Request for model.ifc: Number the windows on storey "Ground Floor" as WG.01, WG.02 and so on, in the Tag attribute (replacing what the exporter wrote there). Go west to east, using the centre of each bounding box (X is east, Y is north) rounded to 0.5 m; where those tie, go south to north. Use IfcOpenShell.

First a look at what the model holds.

```python
import ifcopenshell
import ifcopenshell.util.element
import ifcopenshell.util.placement

model = ifcopenshell.open("model.ifc")
print(model.schema)
storey = next(s for s in model.by_type("IfcBuildingStorey") if s.Name == "Ground Floor")
windows = [e for e in ifcopenshell.util.element.get_decomposition(storey) if e.is_a("IfcWindow")]
for e in sorted(windows, key=lambda e: e.id()):
    origin = ifcopenshell.util.placement.get_local_placement(e.ObjectPlacement)[:3, 3]
    print(e.id(), e.Tag, e.Name, origin.round(2) + 0.0, sep=" | ")
```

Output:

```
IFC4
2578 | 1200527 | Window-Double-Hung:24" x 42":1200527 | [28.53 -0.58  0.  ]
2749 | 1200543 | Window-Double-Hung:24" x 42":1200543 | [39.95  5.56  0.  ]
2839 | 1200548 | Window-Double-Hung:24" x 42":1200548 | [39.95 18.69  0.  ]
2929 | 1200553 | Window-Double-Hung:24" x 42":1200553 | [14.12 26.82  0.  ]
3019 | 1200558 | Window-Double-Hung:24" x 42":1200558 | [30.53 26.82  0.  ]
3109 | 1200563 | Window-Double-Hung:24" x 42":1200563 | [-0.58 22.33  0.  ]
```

```python
import ifcopenshell
import ifcopenshell.geom
import ifcopenshell.util.element
import ifcopenshell.util.shape

model = ifcopenshell.open("model.ifc")
settings = ifcopenshell.geom.settings()
settings.set("use-world-coords", True)


def centre(element):
    shape = ifcopenshell.geom.create_shape(settings, element)
    return ifcopenshell.util.shape.get_bbox_centroid(shape.geometry)


storey = next(s for s in model.by_type("IfcBuildingStorey") if s.Name == "Ground Floor")
windows = [e for e in ifcopenshell.util.element.get_decomposition(storey) if e.is_a("IfcWindow")]

# Insertion points can sit at a corner or the storey origin, so sort by the geometry (in metres).
centres = {e: centre(e) for e in windows}
windows.sort(key=lambda e: (round(centres[e][0] / 0.5), centres[e][1]))

for i, e in enumerate(windows, start=1):
    number = f"WG.{i:02d}"
    e.Tag = number
    print(e.id(), number)

model.write("model_updated.ifc")
```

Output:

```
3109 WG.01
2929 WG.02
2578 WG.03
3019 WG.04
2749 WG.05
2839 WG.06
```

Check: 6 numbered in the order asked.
